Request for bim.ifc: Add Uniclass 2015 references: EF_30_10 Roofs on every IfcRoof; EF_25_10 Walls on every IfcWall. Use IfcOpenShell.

First a look at what the model holds.

```python
import ifcopenshell

model = ifcopenshell.open("bim.ifc")
print(model.schema)
print("classifications:", [c.Name for c in model.by_type("IfcClassification")])
for ifc_class in ("IfcDoor", "IfcRoof", "IfcStair", "IfcWall", "IfcWindow"):
    print(ifc_class, len(model.by_type(ifc_class)))
```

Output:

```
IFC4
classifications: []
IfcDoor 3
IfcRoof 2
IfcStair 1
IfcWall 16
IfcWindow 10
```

```python
import ifcopenshell
import ifcopenshell.api.classification

model = ifcopenshell.open("bim.ifc")

system = ifcopenshell.api.classification.add_classification(model, classification="Uniclass 2015")

codes = {
    "IfcRoof": ("EF_30_10", "Roofs"),
    "IfcWall": ("EF_25_10", "Walls"),
}
for ifc_class, (code, name) in codes.items():
    products = model.by_type(ifc_class)
    ifcopenshell.api.classification.add_reference(
        model, products=products, classification=system, identification=code, name=name
    )
    print(code, len(products))

model.write("bim_rev.ifc")
```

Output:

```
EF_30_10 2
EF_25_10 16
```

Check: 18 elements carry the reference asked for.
